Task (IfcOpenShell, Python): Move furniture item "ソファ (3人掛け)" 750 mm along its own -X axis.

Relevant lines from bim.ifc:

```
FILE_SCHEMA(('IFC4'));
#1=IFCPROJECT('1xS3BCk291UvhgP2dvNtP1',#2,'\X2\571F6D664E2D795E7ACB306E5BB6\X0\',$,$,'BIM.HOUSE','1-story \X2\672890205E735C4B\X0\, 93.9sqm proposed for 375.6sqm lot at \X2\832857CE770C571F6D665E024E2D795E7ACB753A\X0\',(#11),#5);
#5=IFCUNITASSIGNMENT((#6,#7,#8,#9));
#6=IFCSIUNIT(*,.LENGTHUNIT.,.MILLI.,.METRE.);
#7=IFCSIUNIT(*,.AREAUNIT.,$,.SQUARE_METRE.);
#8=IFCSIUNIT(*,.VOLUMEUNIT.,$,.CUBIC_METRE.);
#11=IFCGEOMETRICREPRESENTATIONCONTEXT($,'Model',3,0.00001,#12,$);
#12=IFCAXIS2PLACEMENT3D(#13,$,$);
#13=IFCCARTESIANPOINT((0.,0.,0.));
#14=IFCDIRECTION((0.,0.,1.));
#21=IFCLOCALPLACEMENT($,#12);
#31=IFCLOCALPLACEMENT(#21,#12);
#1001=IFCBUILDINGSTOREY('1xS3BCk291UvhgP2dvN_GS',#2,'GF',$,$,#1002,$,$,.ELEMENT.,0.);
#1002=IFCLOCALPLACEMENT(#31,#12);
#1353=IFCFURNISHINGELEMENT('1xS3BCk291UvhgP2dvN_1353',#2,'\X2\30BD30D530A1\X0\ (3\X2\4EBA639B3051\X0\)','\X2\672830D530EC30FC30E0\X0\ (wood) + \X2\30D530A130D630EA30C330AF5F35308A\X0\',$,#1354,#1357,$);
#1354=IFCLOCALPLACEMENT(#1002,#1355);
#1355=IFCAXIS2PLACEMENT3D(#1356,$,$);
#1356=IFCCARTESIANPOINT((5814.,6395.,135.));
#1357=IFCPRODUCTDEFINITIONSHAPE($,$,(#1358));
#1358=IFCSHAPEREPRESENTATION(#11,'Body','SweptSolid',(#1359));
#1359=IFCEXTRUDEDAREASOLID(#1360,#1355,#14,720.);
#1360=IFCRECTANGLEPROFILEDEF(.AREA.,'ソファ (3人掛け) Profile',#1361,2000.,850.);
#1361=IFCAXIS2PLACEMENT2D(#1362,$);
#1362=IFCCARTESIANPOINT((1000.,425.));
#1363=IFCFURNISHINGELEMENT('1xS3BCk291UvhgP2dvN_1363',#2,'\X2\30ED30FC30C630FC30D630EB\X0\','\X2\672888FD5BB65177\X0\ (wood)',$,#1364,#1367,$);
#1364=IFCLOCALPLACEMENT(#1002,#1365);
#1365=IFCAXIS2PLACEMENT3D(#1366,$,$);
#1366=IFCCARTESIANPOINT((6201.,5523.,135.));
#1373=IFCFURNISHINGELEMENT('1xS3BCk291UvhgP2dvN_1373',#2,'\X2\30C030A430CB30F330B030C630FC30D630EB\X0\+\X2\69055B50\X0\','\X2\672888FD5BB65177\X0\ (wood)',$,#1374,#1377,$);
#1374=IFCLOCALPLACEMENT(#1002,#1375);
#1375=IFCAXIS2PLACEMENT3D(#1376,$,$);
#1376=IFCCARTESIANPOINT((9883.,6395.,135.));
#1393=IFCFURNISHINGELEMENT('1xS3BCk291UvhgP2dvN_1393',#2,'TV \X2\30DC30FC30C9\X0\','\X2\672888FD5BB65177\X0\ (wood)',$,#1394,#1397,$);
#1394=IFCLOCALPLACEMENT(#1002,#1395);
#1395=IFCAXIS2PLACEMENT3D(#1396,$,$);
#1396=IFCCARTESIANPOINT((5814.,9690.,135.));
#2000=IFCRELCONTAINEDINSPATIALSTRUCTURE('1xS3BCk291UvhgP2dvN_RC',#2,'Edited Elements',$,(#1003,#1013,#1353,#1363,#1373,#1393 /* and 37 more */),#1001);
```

```python
import ifcopenshell
import ifcopenshell.api.geometry
import ifcopenshell.util.placement
import ifcopenshell.util.unit

model = ifcopenshell.open("bim.ifc")
unit_scale = ifcopenshell.util.unit.calculate_unit_scale(model)

item = model.by_guid("1xS3BCk291UvhgP2dvN_1353")
matrix = ifcopenshell.util.placement.get_local_placement(item.ObjectPlacement)
matrix[:3, 3] -= matrix[:3, 0] * 0.75 / unit_scale
ifcopenshell.api.geometry.edit_object_placement(model, product=item, matrix=matrix, is_si=False)

print(ifcopenshell.util.placement.get_local_placement(item.ObjectPlacement).round(3) + 0.0)

model.write("bim_updated.ifc")
```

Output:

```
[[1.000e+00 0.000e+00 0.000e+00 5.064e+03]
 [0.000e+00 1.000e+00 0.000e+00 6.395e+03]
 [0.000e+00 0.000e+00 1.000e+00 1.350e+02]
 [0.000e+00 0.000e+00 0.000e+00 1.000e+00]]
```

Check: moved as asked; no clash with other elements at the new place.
